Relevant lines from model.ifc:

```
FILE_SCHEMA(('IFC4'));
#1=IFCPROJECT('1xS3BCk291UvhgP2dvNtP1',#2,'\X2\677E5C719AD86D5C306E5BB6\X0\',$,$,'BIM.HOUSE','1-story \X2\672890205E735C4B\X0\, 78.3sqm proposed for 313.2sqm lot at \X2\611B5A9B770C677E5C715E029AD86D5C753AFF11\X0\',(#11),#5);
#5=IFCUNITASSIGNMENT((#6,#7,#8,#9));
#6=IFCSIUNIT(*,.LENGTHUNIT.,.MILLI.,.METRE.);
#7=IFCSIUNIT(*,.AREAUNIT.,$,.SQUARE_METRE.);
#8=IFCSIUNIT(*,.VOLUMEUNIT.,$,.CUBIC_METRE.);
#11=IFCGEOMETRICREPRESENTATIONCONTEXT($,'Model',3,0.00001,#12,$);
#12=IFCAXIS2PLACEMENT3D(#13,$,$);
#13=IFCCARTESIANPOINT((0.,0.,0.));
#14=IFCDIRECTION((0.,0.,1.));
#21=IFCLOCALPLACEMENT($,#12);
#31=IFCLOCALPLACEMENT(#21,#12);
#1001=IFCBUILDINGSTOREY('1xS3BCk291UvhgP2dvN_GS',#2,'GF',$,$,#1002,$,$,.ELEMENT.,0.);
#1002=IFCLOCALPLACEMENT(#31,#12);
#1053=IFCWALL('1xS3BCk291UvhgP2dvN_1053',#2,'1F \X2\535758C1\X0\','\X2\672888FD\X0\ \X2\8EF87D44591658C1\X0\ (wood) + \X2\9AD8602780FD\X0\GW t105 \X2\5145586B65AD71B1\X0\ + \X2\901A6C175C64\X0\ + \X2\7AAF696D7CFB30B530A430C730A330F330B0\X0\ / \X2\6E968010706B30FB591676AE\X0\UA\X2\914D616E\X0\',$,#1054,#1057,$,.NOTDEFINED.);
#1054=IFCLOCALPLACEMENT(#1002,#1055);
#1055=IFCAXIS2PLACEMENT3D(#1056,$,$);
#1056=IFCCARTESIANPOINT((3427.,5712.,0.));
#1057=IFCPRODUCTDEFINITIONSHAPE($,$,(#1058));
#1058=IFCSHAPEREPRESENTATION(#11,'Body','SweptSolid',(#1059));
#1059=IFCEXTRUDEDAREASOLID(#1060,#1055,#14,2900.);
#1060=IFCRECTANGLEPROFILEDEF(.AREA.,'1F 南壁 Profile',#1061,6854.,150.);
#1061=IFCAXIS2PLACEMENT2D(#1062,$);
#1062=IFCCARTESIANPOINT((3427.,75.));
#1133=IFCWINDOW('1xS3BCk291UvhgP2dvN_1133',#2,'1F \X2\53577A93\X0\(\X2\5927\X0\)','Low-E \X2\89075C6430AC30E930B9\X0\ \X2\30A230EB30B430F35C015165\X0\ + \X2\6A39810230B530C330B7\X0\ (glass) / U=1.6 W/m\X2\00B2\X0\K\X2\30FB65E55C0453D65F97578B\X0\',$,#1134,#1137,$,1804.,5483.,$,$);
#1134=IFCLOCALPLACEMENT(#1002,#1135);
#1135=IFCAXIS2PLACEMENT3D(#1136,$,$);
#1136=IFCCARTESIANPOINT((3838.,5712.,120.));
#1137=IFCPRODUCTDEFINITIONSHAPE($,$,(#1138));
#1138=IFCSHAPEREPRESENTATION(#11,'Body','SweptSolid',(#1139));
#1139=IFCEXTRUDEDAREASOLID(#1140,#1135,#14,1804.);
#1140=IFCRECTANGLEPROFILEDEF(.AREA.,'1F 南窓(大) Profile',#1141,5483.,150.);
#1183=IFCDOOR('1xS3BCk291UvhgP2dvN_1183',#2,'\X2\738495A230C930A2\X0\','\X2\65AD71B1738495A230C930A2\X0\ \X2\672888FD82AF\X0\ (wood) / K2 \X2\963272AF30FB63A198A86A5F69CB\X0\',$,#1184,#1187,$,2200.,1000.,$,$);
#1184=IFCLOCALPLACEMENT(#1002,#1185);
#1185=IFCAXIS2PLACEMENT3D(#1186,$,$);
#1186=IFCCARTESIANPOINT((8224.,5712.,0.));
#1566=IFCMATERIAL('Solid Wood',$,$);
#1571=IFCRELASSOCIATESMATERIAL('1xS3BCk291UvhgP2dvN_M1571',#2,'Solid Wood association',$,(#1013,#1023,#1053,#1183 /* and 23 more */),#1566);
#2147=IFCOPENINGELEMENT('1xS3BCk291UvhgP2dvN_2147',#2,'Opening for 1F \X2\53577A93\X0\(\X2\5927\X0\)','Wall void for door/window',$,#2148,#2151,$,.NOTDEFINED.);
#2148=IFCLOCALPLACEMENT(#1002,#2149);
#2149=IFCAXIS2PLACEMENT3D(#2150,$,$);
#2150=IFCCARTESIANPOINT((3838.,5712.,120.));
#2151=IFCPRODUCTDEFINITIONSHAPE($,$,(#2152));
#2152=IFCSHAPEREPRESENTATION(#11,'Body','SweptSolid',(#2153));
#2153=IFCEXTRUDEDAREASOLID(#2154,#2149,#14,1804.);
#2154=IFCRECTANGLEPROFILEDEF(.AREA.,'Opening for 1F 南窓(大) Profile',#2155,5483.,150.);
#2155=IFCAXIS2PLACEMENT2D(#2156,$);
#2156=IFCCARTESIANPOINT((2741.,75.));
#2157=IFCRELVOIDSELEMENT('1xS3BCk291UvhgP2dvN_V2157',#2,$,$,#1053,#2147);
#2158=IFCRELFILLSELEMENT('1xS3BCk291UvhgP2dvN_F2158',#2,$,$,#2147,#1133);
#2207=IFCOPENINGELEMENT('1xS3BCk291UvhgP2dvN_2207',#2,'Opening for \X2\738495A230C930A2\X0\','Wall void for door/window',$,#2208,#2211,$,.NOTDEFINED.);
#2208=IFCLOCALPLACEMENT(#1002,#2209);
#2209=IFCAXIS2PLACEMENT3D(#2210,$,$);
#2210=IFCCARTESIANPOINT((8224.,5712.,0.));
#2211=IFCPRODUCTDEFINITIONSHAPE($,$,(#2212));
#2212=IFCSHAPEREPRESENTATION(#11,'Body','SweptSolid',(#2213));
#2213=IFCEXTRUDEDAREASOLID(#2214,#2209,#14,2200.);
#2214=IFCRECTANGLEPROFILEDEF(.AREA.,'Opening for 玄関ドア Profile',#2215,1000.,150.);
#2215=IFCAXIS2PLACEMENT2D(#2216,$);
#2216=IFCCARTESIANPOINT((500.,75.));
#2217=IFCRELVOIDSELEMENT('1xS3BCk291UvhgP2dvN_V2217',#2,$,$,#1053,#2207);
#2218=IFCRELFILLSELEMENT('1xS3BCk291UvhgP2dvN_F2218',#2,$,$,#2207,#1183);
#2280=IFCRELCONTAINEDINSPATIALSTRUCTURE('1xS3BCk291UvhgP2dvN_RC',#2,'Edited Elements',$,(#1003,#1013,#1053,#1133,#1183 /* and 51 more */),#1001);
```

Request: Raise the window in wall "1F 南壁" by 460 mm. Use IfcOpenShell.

```python
import numpy as np
import ifcopenshell
import ifcopenshell.api.geometry
import ifcopenshell.util.placement
import ifcopenshell.util.unit

model = ifcopenshell.open("model.ifc")
unit_scale = ifcopenshell.util.unit.calculate_unit_scale(model)

window = model.by_id(1133)
opening = window.FillsVoids[0].RelatingOpeningElement
dz = 460.0

shift = np.array([0.0, 0.0, dz])
# The window is not placed relative to its opening, so move both.
for product in (opening, window):
    matrix = ifcopenshell.util.placement.get_local_placement(product.ObjectPlacement)
    matrix[:3, 3] += shift
    ifcopenshell.api.geometry.edit_object_placement(model, product=product, matrix=matrix, is_si=False)

print(f"moved by {dz * unit_scale:+.3f} m")

model.write("model_updated.ifc")
```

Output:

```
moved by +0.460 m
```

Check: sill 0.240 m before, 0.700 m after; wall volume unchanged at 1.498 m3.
